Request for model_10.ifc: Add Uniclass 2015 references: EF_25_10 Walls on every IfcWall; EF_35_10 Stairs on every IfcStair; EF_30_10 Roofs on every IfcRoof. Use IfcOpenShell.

First a look at what the model holds.

```python
import ifcopenshell

model = ifcopenshell.open("model_10.ifc")
print(model.schema)
print("classifications:", [c.Name for c in model.by_type("IfcClassification")])
for ifc_class in ("IfcDoor", "IfcRoof", "IfcStair", "IfcWall", "IfcWindow"):
    print(ifc_class, len(model.by_type(ifc_class)))
```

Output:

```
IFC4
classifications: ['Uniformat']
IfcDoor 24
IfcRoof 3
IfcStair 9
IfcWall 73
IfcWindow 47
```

```python
import ifcopenshell
import ifcopenshell.api.classification

model = ifcopenshell.open("model_10.ifc")

system = ifcopenshell.api.classification.add_classification(model, classification="Uniclass 2015")

codes = {
    "IfcWall": ("EF_25_10", "Walls"),
    "IfcStair": ("EF_35_10", "Stairs"),
    "IfcRoof": ("EF_30_10", "Roofs"),
}
for ifc_class, (code, name) in codes.items():
    products = model.by_type(ifc_class)
    ifcopenshell.api.classification.add_reference(
        model, products=products, classification=system, identification=code, name=name
    )
    print(code, len(products))

model.write("model_10_edited.ifc")
```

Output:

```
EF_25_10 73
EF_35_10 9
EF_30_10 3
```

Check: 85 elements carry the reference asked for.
